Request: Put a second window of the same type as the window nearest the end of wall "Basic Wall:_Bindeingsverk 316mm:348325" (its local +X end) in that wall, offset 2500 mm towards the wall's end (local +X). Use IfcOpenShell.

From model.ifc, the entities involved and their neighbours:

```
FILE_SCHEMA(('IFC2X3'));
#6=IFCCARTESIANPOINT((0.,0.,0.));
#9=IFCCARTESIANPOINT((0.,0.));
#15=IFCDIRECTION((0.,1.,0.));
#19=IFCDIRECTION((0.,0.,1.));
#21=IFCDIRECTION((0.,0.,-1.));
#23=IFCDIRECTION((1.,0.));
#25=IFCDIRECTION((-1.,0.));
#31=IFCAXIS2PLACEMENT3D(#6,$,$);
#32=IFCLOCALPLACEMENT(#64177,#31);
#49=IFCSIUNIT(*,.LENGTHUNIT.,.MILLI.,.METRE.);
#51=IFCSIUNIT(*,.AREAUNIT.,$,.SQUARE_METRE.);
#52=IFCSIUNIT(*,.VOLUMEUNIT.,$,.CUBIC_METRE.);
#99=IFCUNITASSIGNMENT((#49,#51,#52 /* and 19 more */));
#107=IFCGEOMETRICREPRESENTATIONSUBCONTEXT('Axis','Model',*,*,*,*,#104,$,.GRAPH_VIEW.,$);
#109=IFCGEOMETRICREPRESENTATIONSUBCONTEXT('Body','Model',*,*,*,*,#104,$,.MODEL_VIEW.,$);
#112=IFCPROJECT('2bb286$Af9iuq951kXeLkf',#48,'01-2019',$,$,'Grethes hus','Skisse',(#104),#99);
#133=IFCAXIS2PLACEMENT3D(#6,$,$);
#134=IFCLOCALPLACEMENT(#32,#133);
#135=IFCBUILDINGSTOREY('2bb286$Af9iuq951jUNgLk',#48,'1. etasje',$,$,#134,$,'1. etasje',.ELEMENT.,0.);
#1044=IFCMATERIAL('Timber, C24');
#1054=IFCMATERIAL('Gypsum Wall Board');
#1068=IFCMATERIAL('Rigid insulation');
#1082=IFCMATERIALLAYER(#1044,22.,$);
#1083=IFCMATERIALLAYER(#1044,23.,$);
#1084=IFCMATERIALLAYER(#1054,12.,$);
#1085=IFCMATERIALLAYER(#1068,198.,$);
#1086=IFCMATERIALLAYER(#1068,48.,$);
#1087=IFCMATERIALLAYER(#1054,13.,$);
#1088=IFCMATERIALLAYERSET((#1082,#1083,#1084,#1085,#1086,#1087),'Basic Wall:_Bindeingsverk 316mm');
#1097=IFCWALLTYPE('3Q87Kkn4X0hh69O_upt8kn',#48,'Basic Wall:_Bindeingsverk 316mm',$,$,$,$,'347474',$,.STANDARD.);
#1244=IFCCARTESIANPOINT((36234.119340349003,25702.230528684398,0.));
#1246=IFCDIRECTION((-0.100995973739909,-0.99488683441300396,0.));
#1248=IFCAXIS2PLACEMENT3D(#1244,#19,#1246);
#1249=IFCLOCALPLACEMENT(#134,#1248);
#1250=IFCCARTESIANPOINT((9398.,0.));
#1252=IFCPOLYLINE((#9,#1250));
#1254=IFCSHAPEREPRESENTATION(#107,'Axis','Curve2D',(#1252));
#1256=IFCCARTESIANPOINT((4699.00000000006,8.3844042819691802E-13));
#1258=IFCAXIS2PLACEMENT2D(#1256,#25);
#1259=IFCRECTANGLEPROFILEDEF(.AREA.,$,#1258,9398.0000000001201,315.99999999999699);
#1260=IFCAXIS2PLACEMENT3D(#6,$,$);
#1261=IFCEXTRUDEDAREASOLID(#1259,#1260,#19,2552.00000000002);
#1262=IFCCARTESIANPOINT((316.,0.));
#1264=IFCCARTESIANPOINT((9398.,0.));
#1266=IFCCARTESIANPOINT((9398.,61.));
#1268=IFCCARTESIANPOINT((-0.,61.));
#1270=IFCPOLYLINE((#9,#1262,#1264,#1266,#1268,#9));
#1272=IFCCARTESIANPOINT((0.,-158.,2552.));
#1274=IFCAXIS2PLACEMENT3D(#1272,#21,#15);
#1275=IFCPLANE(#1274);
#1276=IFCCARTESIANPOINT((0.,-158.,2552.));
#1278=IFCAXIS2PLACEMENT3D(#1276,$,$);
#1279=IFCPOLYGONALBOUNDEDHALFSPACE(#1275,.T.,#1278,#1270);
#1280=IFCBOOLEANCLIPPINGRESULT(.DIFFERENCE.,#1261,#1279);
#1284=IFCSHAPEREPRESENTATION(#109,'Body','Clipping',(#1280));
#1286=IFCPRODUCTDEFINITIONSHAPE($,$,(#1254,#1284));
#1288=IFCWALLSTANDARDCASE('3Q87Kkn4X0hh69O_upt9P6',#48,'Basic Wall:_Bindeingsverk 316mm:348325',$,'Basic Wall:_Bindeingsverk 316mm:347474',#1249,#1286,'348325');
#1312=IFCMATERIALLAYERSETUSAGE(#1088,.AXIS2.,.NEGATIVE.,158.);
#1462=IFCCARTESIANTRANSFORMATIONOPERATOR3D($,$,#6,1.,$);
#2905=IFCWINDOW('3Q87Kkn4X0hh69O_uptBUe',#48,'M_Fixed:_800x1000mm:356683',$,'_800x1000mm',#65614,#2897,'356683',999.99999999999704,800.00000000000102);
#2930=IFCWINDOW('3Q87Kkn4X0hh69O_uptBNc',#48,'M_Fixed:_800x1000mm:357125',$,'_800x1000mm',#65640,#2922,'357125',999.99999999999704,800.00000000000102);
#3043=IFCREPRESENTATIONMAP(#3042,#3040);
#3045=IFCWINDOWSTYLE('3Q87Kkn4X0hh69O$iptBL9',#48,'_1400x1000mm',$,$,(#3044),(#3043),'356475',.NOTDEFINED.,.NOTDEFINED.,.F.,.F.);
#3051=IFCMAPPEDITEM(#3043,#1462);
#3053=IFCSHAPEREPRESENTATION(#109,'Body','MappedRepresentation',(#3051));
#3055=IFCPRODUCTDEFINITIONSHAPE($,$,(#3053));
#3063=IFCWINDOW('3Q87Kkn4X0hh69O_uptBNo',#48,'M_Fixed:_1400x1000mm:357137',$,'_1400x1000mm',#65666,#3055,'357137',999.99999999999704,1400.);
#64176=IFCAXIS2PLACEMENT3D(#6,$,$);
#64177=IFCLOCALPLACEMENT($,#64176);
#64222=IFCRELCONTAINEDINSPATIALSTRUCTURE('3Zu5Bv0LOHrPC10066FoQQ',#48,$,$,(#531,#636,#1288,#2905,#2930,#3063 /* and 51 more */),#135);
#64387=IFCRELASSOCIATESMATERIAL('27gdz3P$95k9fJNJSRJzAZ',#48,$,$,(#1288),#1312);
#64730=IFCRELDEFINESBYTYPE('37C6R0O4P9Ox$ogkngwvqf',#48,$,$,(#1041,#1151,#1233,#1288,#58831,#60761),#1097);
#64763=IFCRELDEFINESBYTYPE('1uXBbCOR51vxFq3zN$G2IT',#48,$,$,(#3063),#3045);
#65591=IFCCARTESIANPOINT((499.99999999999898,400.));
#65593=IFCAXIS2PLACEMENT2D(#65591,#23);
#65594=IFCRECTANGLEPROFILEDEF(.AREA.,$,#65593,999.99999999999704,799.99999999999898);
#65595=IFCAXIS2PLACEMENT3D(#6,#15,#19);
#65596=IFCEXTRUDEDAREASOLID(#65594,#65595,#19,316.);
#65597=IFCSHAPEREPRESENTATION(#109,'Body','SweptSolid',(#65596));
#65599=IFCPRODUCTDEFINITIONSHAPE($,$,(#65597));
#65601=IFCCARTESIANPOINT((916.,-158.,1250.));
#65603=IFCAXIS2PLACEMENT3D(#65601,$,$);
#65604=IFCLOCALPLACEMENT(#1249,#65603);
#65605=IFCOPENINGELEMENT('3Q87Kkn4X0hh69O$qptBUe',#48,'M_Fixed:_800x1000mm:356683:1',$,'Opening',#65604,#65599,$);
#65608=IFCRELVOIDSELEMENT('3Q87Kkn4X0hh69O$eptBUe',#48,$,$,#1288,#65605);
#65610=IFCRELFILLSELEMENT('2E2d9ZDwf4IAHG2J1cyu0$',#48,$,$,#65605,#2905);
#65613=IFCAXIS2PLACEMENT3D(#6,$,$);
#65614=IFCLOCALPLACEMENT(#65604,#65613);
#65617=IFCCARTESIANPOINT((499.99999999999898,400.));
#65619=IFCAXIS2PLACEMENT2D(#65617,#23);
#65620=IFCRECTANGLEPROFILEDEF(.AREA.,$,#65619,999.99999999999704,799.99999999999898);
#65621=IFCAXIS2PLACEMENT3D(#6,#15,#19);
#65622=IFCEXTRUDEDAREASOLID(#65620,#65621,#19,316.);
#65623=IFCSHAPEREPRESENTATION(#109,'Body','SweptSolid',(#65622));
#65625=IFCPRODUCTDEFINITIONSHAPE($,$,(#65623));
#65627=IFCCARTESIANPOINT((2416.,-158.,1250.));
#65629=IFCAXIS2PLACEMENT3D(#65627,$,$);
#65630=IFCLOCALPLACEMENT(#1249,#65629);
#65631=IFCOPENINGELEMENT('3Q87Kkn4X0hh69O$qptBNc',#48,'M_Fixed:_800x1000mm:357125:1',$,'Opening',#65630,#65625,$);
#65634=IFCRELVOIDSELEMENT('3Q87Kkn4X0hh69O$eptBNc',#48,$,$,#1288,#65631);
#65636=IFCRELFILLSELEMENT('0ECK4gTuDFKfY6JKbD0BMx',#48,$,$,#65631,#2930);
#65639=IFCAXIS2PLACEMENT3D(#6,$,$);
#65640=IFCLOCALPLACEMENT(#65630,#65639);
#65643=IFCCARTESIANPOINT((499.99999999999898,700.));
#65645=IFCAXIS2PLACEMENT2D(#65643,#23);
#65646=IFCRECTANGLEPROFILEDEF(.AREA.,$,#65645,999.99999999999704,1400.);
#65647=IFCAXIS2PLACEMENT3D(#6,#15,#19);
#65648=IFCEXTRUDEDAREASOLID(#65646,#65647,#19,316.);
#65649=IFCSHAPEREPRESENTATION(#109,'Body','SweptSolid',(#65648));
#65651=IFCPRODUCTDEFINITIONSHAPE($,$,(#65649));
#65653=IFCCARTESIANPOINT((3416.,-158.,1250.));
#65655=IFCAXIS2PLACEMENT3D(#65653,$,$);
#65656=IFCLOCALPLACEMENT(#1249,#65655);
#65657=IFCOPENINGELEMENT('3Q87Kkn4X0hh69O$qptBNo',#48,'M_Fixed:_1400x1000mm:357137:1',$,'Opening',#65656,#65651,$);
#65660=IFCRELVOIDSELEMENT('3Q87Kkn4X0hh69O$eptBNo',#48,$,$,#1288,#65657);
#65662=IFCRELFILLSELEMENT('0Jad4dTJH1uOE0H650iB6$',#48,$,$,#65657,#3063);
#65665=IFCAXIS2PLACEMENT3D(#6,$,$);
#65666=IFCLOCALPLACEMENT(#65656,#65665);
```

```python
import ifcopenshell
import ifcopenshell.api.feature
import ifcopenshell.api.geometry
import ifcopenshell.api.root
import ifcopenshell.geom
import ifcopenshell.util.element
import ifcopenshell.util.placement
import ifcopenshell.util.shape
import ifcopenshell.util.unit

model = ifcopenshell.open("model.ifc")
unit_scale = ifcopenshell.util.unit.calculate_unit_scale(model)
settings = ifcopenshell.geom.settings()


def volume(element):
    """Net volume in cubic metres, openings subtracted."""
    shape = ifcopenshell.geom.create_shape(settings, element)
    return ifcopenshell.util.shape.get_volume(shape.geometry)


def reuse_history(source, copy):
    """copy_class also copies each property set's owner history, people and application; keep the originals."""
    for rel in copy.IsDefinedBy:
        if rel.is_a("IfcRelDefinesByProperties") and (history := rel.RelatingPropertyDefinition.OwnerHistory):
            rel.RelatingPropertyDefinition.OwnerHistory = source.OwnerHistory
            ifcopenshell.util.element.remove_deep2(model, history)


window = model.by_guid("3Q87Kkn4X0hh69O_uptBNo")
opening = window.FillsVoids[0].RelatingOpeningElement
wall = opening.VoidsElements[0].RelatingBuildingElement
before = volume(wall)
shift = ifcopenshell.util.placement.get_local_placement(wall.ObjectPlacement)[:3, 0] * 2.5 / unit_scale

# copy_class copies the void relationship, type, container and properties, but no geometry.
new_opening = ifcopenshell.api.root.copy_class(model, product=opening)
new_opening.Representation = ifcopenshell.util.element.copy_deep(
    model, opening.Representation, exclude=["IfcGeometricRepresentationContext", "IfcRepresentationMap"]
)
new_opening.Name = "M_Fixed:_1400x1000mm"
new_window = ifcopenshell.api.root.copy_class(model, product=window)
new_window.Representation = ifcopenshell.util.element.copy_deep(
    model, window.Representation, exclude=["IfcGeometricRepresentationContext", "IfcRepresentationMap"]
)
new_window.Name = "M_Fixed:_1400x1000mm"
new_window.Tag = None
reuse_history(window, new_window)
fills = ifcopenshell.api.feature.add_filling(model, opening=new_opening, element=new_window)
fills.OwnerHistory = new_window.OwnerHistory  # required in IFC2X3

for old, new in ((opening, new_opening), (window, new_window)):
    matrix = ifcopenshell.util.placement.get_local_placement(old.ObjectPlacement)
    matrix[:3, 3] += shift
    ifcopenshell.api.geometry.edit_object_placement(model, product=new, matrix=matrix, is_si=False)

after = volume(wall)

print(f"wall volume {before:.3f} -> {after:.3f} m3")

model.write("model-out.ifc")
```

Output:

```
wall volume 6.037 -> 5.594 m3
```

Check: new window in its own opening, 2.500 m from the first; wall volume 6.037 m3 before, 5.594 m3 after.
